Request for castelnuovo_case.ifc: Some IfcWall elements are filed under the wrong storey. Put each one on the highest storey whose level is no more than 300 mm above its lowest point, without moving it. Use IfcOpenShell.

First a look at what the model holds.

```python
import ifcopenshell
import ifcopenshell.util.element
import ifcopenshell.util.placement

model = ifcopenshell.open("castelnuovo_case.ifc")
print(model.schema)
for storey in model.by_type("IfcBuildingStorey"):
    level = ifcopenshell.util.placement.get_storey_elevation(storey)
    count = sum(e.is_a("IfcWall") for e in ifcopenshell.util.element.get_contained(storey))
    print(storey.id(), storey.Name, round(level, 3), count, sep=" | ")
```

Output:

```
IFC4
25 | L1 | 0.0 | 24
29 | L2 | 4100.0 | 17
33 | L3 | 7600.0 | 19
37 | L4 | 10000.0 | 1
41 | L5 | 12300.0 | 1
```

```python
import ifcopenshell
import ifcopenshell.api.spatial
import ifcopenshell.geom
import ifcopenshell.util.element
import ifcopenshell.util.placement
import ifcopenshell.util.shape
import ifcopenshell.util.unit

model = ifcopenshell.open("castelnuovo_case.ifc")
unit_scale = ifcopenshell.util.unit.calculate_unit_scale(model)
settings = ifcopenshell.geom.settings()

levels = sorted(
    ((ifcopenshell.util.placement.get_storey_elevation(s) * unit_scale, s) for s in model.by_type("IfcBuildingStorey")),
    key=lambda pair: pair[0],
)

for e in model.by_type("IfcWall"):
    current = e.ContainedInStructure[0].RelatingStructure if e.ContainedInStructure else None
    if current is None or not current.is_a("IfcBuildingStorey"):
        continue
    shape = ifcopenshell.geom.create_shape(settings, e)
    bottom = ifcopenshell.util.shape.get_shape_bottom_elevation(shape, shape.geometry)
    below = [s for level, s in levels if level <= bottom + 0.3]
    storey = below[-1] if below else levels[0][1]
    if storey != current:
        # assign_container keeps the world position.
        ifcopenshell.api.spatial.assign_container(model, products=[e], relating_structure=storey)
        print(e.id(), current.Name, "->", storey.Name)

model.write("castelnuovo_case_edited.ifc")
```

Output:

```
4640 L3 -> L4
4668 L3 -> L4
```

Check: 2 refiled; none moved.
